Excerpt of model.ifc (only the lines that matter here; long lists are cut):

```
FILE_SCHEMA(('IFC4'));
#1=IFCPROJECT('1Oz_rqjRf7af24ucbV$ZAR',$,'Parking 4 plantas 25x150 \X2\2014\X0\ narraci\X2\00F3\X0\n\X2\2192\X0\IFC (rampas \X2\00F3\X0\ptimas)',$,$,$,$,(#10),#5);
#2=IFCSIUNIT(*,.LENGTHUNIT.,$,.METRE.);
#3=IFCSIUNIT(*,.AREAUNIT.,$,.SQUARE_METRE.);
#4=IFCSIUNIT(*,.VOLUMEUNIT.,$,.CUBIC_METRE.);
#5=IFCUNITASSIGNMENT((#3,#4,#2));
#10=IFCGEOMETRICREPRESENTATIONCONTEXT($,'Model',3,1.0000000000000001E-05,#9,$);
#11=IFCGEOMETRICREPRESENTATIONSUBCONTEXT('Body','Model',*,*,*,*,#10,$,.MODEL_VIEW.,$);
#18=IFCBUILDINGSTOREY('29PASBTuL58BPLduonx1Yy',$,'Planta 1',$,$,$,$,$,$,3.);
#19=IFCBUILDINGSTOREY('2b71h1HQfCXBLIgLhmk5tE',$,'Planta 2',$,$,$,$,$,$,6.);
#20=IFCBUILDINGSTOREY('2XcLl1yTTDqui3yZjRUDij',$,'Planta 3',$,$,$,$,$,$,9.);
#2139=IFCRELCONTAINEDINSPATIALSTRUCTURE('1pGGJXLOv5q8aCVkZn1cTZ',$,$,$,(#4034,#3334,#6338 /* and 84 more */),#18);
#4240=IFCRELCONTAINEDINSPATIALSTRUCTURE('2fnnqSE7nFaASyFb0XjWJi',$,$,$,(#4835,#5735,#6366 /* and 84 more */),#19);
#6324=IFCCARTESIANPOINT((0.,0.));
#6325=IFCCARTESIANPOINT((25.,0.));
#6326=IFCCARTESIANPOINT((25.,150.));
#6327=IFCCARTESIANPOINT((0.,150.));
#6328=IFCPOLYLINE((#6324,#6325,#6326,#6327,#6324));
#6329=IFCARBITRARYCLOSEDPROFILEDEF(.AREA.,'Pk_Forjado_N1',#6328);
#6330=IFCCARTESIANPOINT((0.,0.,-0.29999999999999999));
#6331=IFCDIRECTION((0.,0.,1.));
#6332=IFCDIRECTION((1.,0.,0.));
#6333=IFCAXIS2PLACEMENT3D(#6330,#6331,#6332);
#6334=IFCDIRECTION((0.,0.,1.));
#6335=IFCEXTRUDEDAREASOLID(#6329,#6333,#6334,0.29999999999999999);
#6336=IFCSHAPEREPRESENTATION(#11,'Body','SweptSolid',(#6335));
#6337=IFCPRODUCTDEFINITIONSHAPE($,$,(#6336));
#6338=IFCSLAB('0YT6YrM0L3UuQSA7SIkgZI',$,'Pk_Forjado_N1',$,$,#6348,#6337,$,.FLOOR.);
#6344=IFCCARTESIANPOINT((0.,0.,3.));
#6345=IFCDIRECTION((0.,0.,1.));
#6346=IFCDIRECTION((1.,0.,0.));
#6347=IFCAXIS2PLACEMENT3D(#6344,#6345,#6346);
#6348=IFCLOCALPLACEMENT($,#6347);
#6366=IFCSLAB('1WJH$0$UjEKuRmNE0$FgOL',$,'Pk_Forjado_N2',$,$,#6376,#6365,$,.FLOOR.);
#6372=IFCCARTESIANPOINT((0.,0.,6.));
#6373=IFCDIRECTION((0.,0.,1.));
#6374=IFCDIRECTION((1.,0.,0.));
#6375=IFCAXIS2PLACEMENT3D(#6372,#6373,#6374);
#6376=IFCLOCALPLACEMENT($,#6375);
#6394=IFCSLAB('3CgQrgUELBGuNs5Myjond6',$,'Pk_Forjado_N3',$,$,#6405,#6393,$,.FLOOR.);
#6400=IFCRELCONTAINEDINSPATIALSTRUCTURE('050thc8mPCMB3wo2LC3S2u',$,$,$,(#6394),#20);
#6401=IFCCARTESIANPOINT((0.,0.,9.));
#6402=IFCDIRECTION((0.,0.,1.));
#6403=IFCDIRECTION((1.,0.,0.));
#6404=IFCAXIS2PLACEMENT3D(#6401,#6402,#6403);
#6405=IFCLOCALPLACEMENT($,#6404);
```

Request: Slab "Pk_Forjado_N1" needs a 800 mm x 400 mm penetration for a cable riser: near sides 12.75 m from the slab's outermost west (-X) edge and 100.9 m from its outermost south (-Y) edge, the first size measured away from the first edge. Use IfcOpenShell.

```python
import numpy as np
import ifcopenshell
import ifcopenshell.api.feature
import ifcopenshell.api.geometry
import ifcopenshell.api.root
import ifcopenshell.geom
import ifcopenshell.util.placement
import ifcopenshell.util.representation
import ifcopenshell.util.shape
import ifcopenshell.util.unit

model = ifcopenshell.open("model.ifc")
unit_scale = ifcopenshell.util.unit.calculate_unit_scale(model)
settings = ifcopenshell.geom.settings()


def volume(element):
    """Net volume in cubic metres, openings subtracted."""
    shape = ifcopenshell.geom.create_shape(settings, element)
    return ifcopenshell.util.shape.get_volume(shape.geometry)


slab = model.by_guid("0YT6YrM0L3UuQSA7SIkgZI")
before = volume(slab)

# Extent in the slab's own axes, in metres. The edges named are its -X and -Y sides.
slab_shape = ifcopenshell.geom.create_shape(settings, slab)
vertices = ifcopenshell.util.shape.get_vertices(slab_shape.geometry)
x_min, y_min, bottom = vertices.min(axis=0)
top = vertices[:, 2].max()

opening = ifcopenshell.api.root.create_entity(model, ifc_class="IfcOpeningElement", name="Cable riser opening", predefined_type="OPENING")
context = ifcopenshell.util.representation.get_context(model, "Model", "Body", "MODEL_VIEW")
width, depth = 0.8, 0.4
outline = [(0.0, 0.0), (width, 0.0), (width, depth), (0.0, depth), (0.0, 0.0)]
# Overshoot both faces by 50 mm so the cut is clean.
shape = ifcopenshell.api.geometry.add_slab_representation(
    model, context=context, depth=top - bottom + 0.1, polyline=outline
)
ifcopenshell.api.geometry.assign_representation(model, product=opening, representation=shape)

matrix = ifcopenshell.util.placement.get_local_placement(slab.ObjectPlacement)
matrix[:, 3] = matrix @ np.append(np.array([x_min + 12.75, y_min + 100.9, bottom - 0.05]) / unit_scale, 1.0)
ifcopenshell.api.geometry.edit_object_placement(model, product=opening, matrix=matrix, is_si=False)
ifcopenshell.api.feature.add_feature(model, feature=opening, element=slab)

after = volume(slab)

print(f"slab volume {before:.3f} -> {after:.3f} m3")

model.write("model-out.ifc")
```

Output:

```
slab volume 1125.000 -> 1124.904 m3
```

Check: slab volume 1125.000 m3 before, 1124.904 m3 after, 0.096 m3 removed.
